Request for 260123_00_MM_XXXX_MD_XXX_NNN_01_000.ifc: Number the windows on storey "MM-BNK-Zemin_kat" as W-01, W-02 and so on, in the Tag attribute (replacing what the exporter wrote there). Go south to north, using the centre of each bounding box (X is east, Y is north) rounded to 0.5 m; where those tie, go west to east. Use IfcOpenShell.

First a look at what the model holds.

```python
import ifcopenshell
import ifcopenshell.util.element
import ifcopenshell.util.placement

model = ifcopenshell.open("260123_00_MM_XXXX_MD_XXX_NNN_01_000.ifc")
print(model.schema)
storey = next(s for s in model.by_type("IfcBuildingStorey") if s.Name == "MM-BNK-Zemin_kat")
windows = [e for e in ifcopenshell.util.element.get_decomposition(storey) if e.is_a("IfcWindow")]
for e in sorted(windows, key=lambda e: e.id()):
    origin = ifcopenshell.util.placement.get_local_placement(e.ObjectPlacement)[:3, 3]
    print(e.id(), e.Tag, e.Name, origin.round(2) + 0.0, sep=" | ")
```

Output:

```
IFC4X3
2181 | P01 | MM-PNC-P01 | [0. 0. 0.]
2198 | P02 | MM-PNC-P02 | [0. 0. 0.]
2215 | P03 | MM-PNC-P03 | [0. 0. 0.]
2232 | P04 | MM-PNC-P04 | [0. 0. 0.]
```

```python
import ifcopenshell
import ifcopenshell.geom
import ifcopenshell.util.element
import ifcopenshell.util.shape

model = ifcopenshell.open("260123_00_MM_XXXX_MD_XXX_NNN_01_000.ifc")
settings = ifcopenshell.geom.settings()
settings.set("use-world-coords", True)


def centre(element):
    shape = ifcopenshell.geom.create_shape(settings, element)
    return ifcopenshell.util.shape.get_bbox_centroid(shape.geometry)


storey = next(s for s in model.by_type("IfcBuildingStorey") if s.Name == "MM-BNK-Zemin_kat")
windows = [e for e in ifcopenshell.util.element.get_decomposition(storey) if e.is_a("IfcWindow")]

# Insertion points can sit at a corner or the storey origin, so sort by the geometry (in metres).
centres = {e: centre(e) for e in windows}
windows.sort(key=lambda e: (round(centres[e][1] / 0.5), centres[e][0]))

for i, e in enumerate(windows, start=1):
    number = f"W-{i:02d}"
    e.Tag = number
    print(e.id(), number)

model.write("260123_00_MM_XXXX_MD_XXX_NNN_01_000_updated.ifc")
```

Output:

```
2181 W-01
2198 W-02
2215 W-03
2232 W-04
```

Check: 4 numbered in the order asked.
